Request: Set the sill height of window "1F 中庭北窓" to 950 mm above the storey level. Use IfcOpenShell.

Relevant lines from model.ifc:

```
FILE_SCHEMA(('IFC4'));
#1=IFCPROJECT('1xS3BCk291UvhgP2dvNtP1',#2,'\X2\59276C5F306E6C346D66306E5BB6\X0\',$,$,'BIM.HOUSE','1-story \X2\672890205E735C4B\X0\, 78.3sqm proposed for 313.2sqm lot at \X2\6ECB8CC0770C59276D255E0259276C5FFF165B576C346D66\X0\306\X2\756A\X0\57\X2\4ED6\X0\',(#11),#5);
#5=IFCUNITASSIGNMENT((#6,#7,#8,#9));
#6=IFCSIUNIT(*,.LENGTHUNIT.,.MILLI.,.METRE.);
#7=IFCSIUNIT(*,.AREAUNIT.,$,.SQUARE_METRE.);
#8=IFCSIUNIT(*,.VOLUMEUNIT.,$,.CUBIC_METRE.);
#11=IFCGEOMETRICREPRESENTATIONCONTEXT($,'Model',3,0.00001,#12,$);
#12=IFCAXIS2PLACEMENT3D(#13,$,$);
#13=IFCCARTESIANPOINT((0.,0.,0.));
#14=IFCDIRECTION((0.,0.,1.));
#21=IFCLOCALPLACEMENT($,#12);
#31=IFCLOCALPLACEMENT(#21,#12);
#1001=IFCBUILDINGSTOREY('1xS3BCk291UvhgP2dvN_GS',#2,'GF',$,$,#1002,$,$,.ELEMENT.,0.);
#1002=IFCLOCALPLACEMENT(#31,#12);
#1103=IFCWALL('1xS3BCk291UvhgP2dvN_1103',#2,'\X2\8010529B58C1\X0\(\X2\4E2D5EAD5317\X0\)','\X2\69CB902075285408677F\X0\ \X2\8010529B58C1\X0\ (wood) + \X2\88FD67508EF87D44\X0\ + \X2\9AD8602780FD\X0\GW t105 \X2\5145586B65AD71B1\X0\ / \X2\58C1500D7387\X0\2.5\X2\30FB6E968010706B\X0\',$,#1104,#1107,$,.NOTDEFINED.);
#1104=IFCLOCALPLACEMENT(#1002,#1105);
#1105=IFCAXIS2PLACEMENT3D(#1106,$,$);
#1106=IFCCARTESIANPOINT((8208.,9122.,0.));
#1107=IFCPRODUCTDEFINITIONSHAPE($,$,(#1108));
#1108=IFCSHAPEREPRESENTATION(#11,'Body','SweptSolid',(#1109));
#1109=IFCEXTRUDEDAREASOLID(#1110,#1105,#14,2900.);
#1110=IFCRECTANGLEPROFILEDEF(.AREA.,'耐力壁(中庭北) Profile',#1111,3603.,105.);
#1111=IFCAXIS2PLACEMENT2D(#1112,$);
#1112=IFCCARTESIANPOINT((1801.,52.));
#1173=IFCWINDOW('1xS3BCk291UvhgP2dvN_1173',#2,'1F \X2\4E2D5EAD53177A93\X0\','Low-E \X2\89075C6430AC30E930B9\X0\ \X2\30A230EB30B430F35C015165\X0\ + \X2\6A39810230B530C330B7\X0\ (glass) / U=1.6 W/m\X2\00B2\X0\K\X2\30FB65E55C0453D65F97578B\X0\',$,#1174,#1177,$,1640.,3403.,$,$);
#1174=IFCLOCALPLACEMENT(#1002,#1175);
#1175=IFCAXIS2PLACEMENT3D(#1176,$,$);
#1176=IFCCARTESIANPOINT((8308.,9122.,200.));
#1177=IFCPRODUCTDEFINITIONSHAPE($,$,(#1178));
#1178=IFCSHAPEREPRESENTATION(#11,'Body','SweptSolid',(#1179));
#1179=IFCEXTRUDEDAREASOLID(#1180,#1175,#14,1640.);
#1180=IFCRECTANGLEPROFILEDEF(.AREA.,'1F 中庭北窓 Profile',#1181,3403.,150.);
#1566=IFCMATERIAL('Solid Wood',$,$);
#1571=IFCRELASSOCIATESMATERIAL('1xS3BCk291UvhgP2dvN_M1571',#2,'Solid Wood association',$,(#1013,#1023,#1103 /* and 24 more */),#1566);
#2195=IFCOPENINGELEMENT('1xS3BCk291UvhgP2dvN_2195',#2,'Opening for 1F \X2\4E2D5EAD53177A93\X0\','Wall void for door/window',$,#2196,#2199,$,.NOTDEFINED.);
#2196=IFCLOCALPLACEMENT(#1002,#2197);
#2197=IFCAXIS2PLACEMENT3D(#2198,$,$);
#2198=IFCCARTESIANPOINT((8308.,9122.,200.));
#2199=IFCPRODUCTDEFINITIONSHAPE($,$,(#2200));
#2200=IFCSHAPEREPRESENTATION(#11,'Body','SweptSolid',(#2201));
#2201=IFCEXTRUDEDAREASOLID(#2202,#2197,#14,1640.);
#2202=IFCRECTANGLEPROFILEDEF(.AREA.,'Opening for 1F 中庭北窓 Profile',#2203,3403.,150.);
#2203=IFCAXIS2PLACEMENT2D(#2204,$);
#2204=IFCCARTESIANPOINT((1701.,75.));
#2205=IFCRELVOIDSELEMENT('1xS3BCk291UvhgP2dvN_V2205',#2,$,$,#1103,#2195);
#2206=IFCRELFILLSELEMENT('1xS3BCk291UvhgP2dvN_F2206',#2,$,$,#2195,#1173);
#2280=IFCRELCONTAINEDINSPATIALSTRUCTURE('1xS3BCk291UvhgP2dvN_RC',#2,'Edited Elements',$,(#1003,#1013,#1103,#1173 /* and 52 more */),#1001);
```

```python
import numpy as np
import ifcopenshell
import ifcopenshell.api.geometry
import ifcopenshell.geom
import ifcopenshell.util.element
import ifcopenshell.util.placement
import ifcopenshell.util.shape
import ifcopenshell.util.unit

model = ifcopenshell.open("model.ifc")
unit_scale = ifcopenshell.util.unit.calculate_unit_scale(model)

window = model.by_guid("1xS3BCk291UvhgP2dvN_1173")
opening = window.FillsVoids[0].RelatingOpeningElement
storey = ifcopenshell.util.element.get_container(window, ifc_class="IfcBuildingStorey")
level = ifcopenshell.util.placement.get_local_placement(storey.ObjectPlacement)[2, 3]

# The opening's origin need not be at the sill, so measure its lowest point.
shape = ifcopenshell.geom.create_shape(ifcopenshell.geom.settings(), opening)
bottom = ifcopenshell.util.shape.get_shape_bottom_elevation(shape, shape.geometry) / unit_scale
dz = level + 0.95 / unit_scale - bottom

shift = np.array([0.0, 0.0, dz])
# The window is not placed relative to its opening, so move both.
for product in (opening, window):
    matrix = ifcopenshell.util.placement.get_local_placement(product.ObjectPlacement)
    matrix[:3, 3] += shift
    ifcopenshell.api.geometry.edit_object_placement(model, product=product, matrix=matrix, is_si=False)

print(f"moved by {dz * unit_scale:+.3f} m")

model.write("model_updated.ifc")
```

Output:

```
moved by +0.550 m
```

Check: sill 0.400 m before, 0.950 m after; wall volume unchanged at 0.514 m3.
